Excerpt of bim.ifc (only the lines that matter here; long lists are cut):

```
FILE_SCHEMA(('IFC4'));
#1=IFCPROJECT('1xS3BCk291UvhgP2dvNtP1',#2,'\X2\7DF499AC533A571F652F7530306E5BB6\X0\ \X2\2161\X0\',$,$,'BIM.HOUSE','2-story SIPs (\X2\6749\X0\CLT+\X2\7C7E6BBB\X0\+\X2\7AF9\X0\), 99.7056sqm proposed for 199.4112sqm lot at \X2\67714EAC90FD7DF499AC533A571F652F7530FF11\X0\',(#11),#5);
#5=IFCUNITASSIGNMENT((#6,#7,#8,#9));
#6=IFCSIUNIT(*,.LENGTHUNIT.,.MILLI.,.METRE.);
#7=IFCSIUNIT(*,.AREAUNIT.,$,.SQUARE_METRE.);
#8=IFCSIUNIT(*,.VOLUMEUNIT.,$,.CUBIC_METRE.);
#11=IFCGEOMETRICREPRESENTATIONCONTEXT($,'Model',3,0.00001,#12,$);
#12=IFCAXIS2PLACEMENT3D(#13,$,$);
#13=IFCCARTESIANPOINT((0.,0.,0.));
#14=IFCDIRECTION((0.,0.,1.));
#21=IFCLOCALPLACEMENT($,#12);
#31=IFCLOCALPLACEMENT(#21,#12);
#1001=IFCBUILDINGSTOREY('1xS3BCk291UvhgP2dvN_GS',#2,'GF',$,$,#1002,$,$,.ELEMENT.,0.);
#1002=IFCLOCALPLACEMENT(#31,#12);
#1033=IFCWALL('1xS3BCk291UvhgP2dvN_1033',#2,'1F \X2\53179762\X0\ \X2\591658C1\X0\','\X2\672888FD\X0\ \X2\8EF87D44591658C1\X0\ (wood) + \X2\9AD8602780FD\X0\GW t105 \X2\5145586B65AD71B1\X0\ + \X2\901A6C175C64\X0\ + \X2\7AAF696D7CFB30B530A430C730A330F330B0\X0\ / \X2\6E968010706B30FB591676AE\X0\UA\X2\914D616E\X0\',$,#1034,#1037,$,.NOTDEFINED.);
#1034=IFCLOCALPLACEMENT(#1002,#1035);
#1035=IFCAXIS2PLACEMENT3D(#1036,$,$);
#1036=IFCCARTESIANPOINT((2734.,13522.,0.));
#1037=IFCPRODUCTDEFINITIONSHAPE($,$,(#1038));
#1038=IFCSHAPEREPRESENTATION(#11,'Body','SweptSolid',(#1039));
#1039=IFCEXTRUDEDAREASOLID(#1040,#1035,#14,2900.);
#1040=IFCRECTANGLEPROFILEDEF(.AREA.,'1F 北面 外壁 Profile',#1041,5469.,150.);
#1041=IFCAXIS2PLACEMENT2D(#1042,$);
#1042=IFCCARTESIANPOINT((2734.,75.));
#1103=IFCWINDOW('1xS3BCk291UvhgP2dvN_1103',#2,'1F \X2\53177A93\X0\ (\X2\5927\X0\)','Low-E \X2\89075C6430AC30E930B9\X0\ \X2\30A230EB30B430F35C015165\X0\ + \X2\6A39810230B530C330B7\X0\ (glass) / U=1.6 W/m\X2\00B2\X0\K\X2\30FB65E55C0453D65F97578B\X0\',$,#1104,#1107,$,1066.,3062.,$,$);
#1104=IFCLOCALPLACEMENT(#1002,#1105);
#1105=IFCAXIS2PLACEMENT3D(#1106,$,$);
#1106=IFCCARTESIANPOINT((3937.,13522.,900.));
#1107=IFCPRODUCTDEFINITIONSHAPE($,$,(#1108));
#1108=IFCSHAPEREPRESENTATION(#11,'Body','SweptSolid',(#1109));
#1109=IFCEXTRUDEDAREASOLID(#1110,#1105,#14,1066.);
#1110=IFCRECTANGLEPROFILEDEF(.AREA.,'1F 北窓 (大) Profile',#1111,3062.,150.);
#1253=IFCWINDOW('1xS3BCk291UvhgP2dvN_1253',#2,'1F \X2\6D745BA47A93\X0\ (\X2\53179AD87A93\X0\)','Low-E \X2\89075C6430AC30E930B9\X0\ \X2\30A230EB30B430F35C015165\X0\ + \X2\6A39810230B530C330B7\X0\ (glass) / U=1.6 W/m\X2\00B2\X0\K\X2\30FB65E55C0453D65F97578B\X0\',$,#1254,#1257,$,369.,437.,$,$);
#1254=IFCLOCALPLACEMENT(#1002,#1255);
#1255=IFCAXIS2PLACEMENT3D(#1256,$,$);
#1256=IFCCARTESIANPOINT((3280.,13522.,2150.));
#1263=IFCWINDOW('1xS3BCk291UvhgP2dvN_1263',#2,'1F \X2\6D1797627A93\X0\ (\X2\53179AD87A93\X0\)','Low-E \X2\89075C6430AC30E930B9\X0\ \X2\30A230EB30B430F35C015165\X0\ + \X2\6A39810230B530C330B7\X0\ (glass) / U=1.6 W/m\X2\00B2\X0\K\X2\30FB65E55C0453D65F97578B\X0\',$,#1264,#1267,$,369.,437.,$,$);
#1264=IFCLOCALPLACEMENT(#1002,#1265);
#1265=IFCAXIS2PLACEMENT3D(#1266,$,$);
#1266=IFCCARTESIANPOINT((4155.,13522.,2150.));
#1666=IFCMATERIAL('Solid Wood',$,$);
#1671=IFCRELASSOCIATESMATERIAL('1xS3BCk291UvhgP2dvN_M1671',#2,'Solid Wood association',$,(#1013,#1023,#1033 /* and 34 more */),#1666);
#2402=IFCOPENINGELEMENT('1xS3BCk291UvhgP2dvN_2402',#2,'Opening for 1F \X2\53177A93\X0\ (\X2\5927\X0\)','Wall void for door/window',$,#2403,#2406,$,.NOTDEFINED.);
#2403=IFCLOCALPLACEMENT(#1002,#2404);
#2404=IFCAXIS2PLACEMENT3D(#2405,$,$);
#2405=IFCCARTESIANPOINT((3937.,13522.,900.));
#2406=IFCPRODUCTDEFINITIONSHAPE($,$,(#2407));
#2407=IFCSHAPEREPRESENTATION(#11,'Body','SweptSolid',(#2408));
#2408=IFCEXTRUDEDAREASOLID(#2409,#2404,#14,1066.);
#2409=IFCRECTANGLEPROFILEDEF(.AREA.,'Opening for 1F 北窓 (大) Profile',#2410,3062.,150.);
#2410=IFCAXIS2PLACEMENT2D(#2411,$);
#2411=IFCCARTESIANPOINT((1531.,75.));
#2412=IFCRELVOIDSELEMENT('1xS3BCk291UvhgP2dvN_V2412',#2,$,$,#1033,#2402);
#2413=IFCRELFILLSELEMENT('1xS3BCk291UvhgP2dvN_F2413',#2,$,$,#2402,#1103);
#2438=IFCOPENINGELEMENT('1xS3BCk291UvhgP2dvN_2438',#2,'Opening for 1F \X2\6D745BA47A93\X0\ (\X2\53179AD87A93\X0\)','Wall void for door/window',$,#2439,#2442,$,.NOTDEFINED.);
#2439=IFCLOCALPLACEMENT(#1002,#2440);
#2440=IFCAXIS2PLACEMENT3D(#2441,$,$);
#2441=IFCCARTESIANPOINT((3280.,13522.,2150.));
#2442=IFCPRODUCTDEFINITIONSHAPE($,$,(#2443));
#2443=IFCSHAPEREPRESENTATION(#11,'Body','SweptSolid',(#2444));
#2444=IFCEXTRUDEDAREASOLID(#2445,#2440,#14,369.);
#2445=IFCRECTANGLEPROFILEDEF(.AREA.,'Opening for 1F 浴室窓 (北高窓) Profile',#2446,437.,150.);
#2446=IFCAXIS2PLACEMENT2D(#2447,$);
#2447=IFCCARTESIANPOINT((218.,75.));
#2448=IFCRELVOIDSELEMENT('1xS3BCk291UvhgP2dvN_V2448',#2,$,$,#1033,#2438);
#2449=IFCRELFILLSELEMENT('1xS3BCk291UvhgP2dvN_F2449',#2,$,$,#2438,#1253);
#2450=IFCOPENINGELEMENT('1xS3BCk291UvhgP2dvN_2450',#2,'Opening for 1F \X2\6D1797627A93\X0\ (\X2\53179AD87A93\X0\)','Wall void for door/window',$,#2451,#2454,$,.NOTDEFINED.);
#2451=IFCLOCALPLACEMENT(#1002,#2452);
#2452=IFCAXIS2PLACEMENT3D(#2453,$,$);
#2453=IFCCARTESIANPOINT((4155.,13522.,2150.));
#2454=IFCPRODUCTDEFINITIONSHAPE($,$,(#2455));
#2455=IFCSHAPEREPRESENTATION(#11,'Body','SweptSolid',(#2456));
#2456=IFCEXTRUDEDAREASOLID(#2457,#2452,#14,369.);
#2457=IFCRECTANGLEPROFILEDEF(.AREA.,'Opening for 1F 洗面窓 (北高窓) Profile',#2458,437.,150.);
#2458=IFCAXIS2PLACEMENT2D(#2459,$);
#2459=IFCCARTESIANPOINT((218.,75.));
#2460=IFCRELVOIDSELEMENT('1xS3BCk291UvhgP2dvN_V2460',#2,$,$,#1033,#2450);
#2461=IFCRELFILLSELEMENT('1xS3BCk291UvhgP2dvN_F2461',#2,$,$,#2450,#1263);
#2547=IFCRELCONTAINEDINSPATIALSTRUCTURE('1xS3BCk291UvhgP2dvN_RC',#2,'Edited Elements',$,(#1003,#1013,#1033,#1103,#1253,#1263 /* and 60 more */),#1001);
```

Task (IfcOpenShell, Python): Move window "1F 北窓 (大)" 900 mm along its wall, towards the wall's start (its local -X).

```python
import ifcopenshell
import ifcopenshell.api.geometry
import ifcopenshell.util.placement
import ifcopenshell.util.unit

model = ifcopenshell.open("bim.ifc")
unit_scale = ifcopenshell.util.unit.calculate_unit_scale(model)

window = model.by_guid("1xS3BCk291UvhgP2dvN_1103")
opening = window.FillsVoids[0].RelatingOpeningElement
wall = opening.VoidsElements[0].RelatingBuildingElement

wall_matrix = ifcopenshell.util.placement.get_local_placement(wall.ObjectPlacement)
shift = wall_matrix[:3, 0] * -0.9 / unit_scale
before = ifcopenshell.util.placement.get_local_placement(window.ObjectPlacement)[:3, 3].copy()

# The window is not placed relative to its opening, so move both.
for product in (opening, window):
    matrix = ifcopenshell.util.placement.get_local_placement(product.ObjectPlacement)
    matrix[:3, 3] += shift
    ifcopenshell.api.geometry.edit_object_placement(model, product=product, matrix=matrix, is_si=False)

after = ifcopenshell.util.placement.get_local_placement(window.ObjectPlacement)[:3, 3]
print("window moved by", (after - before).round(3) + 0.0)

model.write("bim_rev.ifc")
```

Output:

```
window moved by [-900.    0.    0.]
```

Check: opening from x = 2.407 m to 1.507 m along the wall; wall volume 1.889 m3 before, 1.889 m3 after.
